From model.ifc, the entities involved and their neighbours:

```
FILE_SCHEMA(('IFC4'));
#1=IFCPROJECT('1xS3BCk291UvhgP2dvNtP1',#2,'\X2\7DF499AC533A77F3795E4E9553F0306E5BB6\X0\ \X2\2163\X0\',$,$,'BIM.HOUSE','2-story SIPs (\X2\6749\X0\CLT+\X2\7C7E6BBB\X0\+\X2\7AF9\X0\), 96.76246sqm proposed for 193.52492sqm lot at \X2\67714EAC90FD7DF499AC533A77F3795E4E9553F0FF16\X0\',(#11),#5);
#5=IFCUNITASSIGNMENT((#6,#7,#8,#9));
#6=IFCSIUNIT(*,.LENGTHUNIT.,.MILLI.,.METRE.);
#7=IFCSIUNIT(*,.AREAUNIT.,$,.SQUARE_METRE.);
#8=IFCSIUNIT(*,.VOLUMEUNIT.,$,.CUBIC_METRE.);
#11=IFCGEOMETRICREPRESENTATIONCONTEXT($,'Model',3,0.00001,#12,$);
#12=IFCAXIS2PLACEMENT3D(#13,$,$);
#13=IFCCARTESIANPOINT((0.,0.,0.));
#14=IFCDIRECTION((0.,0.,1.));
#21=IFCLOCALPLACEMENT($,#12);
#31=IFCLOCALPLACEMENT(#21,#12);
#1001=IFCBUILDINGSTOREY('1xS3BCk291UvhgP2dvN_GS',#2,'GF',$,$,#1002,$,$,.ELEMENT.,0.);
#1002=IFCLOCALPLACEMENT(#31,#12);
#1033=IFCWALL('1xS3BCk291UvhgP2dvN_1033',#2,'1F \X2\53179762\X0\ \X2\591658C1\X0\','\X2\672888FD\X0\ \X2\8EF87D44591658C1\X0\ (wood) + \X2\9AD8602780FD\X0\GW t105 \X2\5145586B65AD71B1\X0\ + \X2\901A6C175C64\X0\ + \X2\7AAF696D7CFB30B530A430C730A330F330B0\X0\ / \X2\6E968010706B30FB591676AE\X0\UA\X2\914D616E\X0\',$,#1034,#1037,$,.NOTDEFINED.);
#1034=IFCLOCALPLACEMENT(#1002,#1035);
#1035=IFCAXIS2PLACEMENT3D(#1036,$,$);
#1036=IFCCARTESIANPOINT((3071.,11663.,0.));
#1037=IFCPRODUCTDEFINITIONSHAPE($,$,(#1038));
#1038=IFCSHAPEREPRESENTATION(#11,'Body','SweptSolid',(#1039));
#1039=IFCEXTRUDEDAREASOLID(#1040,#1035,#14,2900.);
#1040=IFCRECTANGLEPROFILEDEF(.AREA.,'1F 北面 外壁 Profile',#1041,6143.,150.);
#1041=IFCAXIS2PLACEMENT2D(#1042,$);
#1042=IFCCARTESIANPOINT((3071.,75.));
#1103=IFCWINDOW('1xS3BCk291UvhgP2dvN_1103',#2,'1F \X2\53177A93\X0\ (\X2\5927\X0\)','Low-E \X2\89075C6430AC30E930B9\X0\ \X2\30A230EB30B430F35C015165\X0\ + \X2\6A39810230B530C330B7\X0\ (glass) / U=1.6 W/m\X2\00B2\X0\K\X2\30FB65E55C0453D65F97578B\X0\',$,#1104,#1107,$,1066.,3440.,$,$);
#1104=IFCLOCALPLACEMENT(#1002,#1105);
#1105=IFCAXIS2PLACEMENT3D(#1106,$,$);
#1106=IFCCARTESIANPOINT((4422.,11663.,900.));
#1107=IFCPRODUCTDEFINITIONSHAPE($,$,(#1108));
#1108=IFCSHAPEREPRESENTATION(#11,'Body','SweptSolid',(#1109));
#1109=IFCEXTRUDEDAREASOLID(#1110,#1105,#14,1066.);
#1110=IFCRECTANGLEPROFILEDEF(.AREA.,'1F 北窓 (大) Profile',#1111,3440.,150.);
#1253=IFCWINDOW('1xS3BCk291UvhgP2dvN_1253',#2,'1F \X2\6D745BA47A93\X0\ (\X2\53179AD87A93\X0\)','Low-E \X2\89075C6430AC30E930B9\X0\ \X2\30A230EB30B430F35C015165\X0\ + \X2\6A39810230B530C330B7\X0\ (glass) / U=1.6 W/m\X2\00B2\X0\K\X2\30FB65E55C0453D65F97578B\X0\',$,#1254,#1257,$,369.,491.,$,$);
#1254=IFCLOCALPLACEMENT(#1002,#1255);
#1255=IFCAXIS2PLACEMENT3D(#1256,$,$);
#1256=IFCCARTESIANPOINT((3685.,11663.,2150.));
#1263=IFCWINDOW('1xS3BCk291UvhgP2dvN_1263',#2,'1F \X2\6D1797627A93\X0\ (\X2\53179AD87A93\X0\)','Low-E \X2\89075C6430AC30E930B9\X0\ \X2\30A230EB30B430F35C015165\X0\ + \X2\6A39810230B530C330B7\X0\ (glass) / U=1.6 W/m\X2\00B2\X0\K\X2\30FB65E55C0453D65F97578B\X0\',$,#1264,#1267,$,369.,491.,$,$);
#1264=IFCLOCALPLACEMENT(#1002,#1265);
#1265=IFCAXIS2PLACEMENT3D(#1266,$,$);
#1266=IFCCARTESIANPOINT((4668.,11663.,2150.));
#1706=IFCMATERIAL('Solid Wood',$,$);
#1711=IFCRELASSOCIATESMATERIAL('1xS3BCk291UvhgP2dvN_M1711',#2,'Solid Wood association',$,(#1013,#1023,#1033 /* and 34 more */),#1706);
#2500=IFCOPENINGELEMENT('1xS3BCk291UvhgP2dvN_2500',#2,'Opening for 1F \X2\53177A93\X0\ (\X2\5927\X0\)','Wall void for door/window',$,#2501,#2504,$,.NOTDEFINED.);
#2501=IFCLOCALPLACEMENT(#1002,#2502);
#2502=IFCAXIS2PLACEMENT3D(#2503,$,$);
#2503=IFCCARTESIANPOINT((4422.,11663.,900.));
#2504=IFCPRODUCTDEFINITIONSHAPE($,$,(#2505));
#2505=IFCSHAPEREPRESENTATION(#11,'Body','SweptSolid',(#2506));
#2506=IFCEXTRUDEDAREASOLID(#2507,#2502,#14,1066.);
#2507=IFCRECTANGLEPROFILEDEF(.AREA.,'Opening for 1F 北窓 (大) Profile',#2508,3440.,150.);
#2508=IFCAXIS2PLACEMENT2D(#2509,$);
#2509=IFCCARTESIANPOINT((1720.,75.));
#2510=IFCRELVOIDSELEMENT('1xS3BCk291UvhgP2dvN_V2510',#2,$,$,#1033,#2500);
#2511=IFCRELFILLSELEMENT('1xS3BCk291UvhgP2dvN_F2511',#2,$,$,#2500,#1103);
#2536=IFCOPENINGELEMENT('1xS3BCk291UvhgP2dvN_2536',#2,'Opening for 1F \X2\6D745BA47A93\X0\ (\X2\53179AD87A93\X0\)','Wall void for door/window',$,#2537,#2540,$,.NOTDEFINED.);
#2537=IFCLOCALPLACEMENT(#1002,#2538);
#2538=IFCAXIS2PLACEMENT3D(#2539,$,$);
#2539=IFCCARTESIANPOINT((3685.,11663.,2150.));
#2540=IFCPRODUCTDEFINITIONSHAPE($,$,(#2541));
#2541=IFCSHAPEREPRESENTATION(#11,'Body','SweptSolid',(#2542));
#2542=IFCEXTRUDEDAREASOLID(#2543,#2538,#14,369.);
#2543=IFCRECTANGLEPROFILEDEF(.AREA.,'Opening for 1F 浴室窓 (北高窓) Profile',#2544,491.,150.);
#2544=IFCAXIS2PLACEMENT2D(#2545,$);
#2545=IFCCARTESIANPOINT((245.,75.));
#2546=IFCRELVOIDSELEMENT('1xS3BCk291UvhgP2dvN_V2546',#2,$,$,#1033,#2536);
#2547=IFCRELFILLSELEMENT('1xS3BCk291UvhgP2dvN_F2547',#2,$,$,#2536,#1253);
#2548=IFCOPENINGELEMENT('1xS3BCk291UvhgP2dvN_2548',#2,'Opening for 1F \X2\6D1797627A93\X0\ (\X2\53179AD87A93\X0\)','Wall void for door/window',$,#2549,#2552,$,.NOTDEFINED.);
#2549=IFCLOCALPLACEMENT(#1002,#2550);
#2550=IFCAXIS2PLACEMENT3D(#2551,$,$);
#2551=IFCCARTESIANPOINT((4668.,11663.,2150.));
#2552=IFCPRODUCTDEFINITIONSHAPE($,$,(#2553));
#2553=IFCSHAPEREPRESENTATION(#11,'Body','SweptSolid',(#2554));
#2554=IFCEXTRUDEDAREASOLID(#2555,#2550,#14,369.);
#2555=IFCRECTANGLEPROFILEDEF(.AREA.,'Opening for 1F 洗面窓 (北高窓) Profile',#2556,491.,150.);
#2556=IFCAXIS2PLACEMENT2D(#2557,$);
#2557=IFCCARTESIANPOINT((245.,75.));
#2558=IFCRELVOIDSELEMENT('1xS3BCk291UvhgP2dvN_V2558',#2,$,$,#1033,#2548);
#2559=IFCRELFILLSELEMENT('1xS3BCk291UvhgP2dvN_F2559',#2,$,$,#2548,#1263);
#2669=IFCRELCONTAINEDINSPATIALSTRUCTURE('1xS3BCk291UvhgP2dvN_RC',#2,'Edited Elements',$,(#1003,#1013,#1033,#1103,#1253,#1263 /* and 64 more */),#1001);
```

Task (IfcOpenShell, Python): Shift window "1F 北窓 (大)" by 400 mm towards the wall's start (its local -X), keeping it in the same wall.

```python
import ifcopenshell
import ifcopenshell.api.geometry
import ifcopenshell.util.placement
import ifcopenshell.util.unit

model = ifcopenshell.open("model.ifc")
unit_scale = ifcopenshell.util.unit.calculate_unit_scale(model)

window = model.by_guid("1xS3BCk291UvhgP2dvN_1103")
opening = window.FillsVoids[0].RelatingOpeningElement
wall = opening.VoidsElements[0].RelatingBuildingElement

wall_matrix = ifcopenshell.util.placement.get_local_placement(wall.ObjectPlacement)
shift = wall_matrix[:3, 0] * -0.4 / unit_scale
before = ifcopenshell.util.placement.get_local_placement(window.ObjectPlacement)[:3, 3].copy()

# The window is not placed relative to its opening, so move both.
for product in (opening, window):
    matrix = ifcopenshell.util.placement.get_local_placement(product.ObjectPlacement)
    matrix[:3, 3] += shift
    ifcopenshell.api.geometry.edit_object_placement(model, product=product, matrix=matrix, is_si=False)

after = ifcopenshell.util.placement.get_local_placement(window.ObjectPlacement)[:3, 3]
print("window moved by", (after - before).round(3) + 0.0)

model.write("model_edited.ifc")
```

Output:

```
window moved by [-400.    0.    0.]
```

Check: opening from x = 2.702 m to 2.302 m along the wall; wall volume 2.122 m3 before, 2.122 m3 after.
